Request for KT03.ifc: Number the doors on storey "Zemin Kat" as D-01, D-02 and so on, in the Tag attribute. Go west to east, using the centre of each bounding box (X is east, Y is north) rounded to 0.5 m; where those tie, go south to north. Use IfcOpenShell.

First a look at what the model holds.

```python
import ifcopenshell
import ifcopenshell.util.element
import ifcopenshell.util.placement

model = ifcopenshell.open("KT03.ifc")
print(model.schema)
storey = next(s for s in model.by_type("IfcBuildingStorey") if s.Name == "Zemin Kat")
doors = [e for e in ifcopenshell.util.element.get_decomposition(storey) if e.is_a("IfcDoor")]
for e in sorted(doors, key=lambda e: e.id()):
    origin = ifcopenshell.util.placement.get_local_placement(e.ObjectPlacement)[:3, 3]
    print(e.id(), e.Tag, e.Name, origin.round(2) + 0.0, sep=" | ")
```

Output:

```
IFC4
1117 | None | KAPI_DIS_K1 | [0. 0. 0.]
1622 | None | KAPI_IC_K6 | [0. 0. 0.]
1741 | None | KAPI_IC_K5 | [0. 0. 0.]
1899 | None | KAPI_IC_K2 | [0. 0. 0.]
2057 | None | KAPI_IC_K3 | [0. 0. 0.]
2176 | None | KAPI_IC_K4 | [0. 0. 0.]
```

```python
import ifcopenshell
import ifcopenshell.geom
import ifcopenshell.util.element
import ifcopenshell.util.shape

model = ifcopenshell.open("KT03.ifc")
settings = ifcopenshell.geom.settings()
settings.set("use-world-coords", True)


def centre(element):
    shape = ifcopenshell.geom.create_shape(settings, element)
    return ifcopenshell.util.shape.get_bbox_centroid(shape.geometry)


storey = next(s for s in model.by_type("IfcBuildingStorey") if s.Name == "Zemin Kat")
doors = [e for e in ifcopenshell.util.element.get_decomposition(storey) if e.is_a("IfcDoor")]

# Insertion points can sit at a corner or the storey origin, so sort by the geometry (in metres).
centres = {e: centre(e) for e in doors}
doors.sort(key=lambda e: (round(centres[e][0] / 0.5), centres[e][1]))

for i, e in enumerate(doors, start=1):
    number = f"D-{i:02d}"
    e.Tag = number
    print(e.id(), number)

model.write("KT03_updated.ifc")
```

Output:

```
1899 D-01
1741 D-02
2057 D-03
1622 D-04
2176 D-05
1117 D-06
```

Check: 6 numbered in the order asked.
